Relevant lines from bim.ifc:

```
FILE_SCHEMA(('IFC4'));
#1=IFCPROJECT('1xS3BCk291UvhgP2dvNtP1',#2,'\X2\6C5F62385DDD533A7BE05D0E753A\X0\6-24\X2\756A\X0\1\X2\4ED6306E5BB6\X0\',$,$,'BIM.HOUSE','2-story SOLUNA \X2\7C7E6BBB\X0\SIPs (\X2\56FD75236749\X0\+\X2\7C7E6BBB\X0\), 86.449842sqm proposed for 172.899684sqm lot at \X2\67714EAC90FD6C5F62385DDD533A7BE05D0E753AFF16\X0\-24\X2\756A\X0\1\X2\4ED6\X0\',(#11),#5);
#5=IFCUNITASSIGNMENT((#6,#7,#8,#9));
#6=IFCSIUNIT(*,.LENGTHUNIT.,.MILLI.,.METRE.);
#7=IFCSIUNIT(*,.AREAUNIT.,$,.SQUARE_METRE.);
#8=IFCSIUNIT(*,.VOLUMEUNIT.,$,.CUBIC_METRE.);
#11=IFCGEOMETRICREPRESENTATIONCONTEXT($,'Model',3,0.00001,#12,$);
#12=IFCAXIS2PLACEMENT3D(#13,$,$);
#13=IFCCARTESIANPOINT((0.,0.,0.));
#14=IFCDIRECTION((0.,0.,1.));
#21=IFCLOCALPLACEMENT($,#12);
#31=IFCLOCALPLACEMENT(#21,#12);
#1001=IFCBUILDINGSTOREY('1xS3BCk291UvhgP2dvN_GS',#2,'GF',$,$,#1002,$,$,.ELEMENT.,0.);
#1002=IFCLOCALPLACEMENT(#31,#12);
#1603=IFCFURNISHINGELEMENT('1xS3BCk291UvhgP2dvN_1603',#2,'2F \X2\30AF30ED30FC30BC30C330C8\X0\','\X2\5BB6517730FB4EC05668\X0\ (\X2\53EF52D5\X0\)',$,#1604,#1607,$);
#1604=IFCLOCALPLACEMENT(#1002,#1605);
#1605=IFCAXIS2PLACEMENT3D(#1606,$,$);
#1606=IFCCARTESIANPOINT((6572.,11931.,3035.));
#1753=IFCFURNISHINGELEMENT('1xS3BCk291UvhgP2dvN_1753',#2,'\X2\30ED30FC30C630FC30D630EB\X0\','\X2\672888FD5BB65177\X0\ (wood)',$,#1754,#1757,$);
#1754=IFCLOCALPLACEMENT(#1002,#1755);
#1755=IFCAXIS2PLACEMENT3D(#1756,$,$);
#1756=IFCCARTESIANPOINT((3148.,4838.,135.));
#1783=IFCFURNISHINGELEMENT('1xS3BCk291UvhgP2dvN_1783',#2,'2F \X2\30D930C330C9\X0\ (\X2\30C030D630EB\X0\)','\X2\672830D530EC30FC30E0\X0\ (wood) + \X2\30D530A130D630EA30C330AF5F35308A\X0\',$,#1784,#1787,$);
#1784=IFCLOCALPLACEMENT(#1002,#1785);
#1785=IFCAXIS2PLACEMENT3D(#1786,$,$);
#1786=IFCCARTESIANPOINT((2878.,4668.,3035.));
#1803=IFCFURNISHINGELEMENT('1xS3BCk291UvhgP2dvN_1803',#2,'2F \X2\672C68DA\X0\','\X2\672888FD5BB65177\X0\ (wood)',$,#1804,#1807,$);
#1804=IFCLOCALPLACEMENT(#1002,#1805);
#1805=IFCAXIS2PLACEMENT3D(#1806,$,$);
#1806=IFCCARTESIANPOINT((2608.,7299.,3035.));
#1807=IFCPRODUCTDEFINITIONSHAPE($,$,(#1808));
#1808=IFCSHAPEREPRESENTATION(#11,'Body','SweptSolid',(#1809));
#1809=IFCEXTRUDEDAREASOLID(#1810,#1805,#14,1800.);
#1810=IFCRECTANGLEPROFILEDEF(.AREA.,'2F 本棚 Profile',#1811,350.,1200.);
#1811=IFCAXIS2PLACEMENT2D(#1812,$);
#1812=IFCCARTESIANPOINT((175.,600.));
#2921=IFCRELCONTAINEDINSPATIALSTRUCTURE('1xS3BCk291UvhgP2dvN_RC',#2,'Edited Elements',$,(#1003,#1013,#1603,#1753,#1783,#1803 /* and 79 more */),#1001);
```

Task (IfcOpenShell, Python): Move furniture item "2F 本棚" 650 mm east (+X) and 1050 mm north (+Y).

```python
import ifcopenshell
import ifcopenshell.api.geometry
import ifcopenshell.util.placement
import ifcopenshell.util.unit

model = ifcopenshell.open("bim.ifc")
unit_scale = ifcopenshell.util.unit.calculate_unit_scale(model)

item = model.by_guid("1xS3BCk291UvhgP2dvN_1803")
matrix = ifcopenshell.util.placement.get_local_placement(item.ObjectPlacement)
matrix[0, 3] += 0.65 / unit_scale
matrix[1, 3] += 1.05 / unit_scale
ifcopenshell.api.geometry.edit_object_placement(model, product=item, matrix=matrix, is_si=False)

print(ifcopenshell.util.placement.get_local_placement(item.ObjectPlacement).round(3) + 0.0)

model.write("bim_v2.ifc")
```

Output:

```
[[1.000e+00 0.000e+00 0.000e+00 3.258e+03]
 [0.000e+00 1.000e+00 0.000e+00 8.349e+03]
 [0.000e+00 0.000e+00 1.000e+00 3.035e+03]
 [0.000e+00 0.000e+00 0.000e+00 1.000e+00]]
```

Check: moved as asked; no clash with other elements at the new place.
